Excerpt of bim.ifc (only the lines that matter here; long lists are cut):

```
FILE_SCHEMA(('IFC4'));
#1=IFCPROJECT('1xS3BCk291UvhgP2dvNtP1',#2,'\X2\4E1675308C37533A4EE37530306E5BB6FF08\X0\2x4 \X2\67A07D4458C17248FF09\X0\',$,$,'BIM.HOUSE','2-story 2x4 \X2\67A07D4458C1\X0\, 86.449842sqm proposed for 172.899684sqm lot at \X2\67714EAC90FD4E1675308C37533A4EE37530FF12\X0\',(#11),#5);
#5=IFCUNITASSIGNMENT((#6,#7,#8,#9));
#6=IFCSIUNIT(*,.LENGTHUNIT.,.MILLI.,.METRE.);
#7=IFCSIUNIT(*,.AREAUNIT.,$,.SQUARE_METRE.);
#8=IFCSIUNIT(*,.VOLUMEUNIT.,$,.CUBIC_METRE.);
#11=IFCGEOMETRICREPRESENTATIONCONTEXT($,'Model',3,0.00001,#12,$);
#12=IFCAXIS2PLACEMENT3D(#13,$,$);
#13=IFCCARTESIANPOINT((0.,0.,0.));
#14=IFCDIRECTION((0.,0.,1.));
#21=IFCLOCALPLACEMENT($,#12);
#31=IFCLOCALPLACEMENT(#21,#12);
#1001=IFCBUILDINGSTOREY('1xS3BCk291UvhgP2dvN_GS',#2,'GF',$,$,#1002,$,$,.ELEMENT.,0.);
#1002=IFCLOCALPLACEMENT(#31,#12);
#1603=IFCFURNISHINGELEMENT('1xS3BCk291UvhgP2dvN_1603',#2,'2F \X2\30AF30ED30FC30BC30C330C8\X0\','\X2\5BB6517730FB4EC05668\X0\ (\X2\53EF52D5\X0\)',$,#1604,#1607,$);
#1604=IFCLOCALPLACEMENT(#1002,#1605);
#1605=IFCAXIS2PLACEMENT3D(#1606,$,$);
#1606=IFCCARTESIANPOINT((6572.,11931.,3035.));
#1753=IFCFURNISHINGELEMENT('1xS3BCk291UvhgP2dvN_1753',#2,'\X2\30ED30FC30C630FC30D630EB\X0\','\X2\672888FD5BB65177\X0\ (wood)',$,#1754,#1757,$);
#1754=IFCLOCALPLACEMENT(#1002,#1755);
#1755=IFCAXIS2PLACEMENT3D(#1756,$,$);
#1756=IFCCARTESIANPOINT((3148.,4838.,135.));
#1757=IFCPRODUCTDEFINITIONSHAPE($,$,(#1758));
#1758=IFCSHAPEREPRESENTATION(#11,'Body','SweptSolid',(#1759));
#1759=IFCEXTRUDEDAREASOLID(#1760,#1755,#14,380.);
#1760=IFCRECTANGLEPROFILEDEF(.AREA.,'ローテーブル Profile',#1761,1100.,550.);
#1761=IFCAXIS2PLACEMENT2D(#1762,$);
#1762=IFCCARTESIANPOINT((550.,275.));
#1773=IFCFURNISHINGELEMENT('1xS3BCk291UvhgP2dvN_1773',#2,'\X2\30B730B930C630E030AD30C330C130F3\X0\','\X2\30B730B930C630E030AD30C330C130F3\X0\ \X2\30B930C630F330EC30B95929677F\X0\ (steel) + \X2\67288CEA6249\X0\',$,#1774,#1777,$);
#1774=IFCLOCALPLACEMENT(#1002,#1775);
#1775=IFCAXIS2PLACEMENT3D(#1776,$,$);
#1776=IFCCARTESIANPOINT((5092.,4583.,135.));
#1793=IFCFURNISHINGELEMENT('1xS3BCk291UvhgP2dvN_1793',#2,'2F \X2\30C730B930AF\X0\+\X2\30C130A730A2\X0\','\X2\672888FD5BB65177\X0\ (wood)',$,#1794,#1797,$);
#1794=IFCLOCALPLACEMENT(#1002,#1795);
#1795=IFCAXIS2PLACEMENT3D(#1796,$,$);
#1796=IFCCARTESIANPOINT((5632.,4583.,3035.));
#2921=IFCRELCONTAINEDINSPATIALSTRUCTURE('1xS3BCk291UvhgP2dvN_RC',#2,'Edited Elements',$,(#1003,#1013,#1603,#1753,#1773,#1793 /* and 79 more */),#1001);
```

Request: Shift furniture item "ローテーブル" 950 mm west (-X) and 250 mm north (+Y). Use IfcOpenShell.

```python
import ifcopenshell
import ifcopenshell.api.geometry
import ifcopenshell.util.placement

model = ifcopenshell.open("bim.ifc")

item = model.by_guid("1xS3BCk291UvhgP2dvN_1753")
matrix = ifcopenshell.util.placement.get_local_placement(item.ObjectPlacement)
matrix[0, 3] -= 950.0
matrix[1, 3] += 250.0
ifcopenshell.api.geometry.edit_object_placement(model, product=item, matrix=matrix, is_si=False)

print(ifcopenshell.util.placement.get_local_placement(item.ObjectPlacement).round(3) + 0.0)

model.write("bim_updated.ifc")
```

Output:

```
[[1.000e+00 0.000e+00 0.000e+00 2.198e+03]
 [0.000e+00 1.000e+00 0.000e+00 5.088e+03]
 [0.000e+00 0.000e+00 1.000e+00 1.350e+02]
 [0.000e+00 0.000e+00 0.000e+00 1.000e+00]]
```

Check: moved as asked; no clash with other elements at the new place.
